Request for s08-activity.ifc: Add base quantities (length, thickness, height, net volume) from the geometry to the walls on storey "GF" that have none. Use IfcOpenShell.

First a look at what the model holds.

```python
import ifcopenshell
import ifcopenshell.util.element
import ifcopenshell.util.unit

model = ifcopenshell.open("s08-activity.ifc")
print(model.schema)
for unit_type in ("LENGTHUNIT", "AREAUNIT", "VOLUMEUNIT"):
    print(unit_type, ifcopenshell.util.unit.calculate_unit_scale(model, unit_type))
storey = next(s for s in model.by_type("IfcBuildingStorey") if s.Name == "GF")
walls = [e for e in ifcopenshell.util.element.get_decomposition(storey) if e.is_a("IfcWall")]
for e in sorted(walls, key=lambda e: e.id()):
    print(e.id(), e.is_a(), e.Name, list(ifcopenshell.util.element.get_psets(e, qtos_only=True)), sep=" | ")
```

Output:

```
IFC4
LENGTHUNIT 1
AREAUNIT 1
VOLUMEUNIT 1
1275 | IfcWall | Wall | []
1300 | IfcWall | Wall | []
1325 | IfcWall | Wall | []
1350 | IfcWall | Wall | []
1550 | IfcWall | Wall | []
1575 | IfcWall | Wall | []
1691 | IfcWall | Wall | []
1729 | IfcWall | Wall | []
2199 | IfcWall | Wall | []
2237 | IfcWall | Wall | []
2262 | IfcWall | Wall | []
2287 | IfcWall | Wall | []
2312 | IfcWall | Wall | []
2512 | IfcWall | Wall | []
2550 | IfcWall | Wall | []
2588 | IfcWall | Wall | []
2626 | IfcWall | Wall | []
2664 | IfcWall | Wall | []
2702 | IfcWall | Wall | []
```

```python
import ifcopenshell
import ifcopenshell.api.pset
import ifcopenshell.geom
import ifcopenshell.util.element
import ifcopenshell.util.shape
import ifcopenshell.util.unit

model = ifcopenshell.open("s08-activity.ifc")
unit_scale = ifcopenshell.util.unit.calculate_unit_scale(model)
volume_scale = ifcopenshell.util.unit.calculate_unit_scale(model, "VOLUMEUNIT")
settings = ifcopenshell.geom.settings()

storey = next(s for s in model.by_type("IfcBuildingStorey") if s.Name == "GF")
walls = [e for e in ifcopenshell.util.element.get_decomposition(storey) if e.is_a("IfcWall")]

for e in sorted(walls, key=lambda e: e.id()):
    if ifcopenshell.util.element.get_psets(e, qtos_only=True, should_inherit=False):
        continue
    # Geometry comes back in metres, in the element's own axes.
    shape = ifcopenshell.geom.create_shape(settings, e)
    values = {
        "Length": ifcopenshell.util.shape.get_x(shape.geometry) / unit_scale,
        "Width": ifcopenshell.util.shape.get_y(shape.geometry) / unit_scale,
        "Height": ifcopenshell.util.shape.get_z(shape.geometry) / unit_scale,
        "NetVolume": ifcopenshell.util.shape.get_volume(shape.geometry) / volume_scale,
    }
    qto = ifcopenshell.api.pset.add_qto(model, product=e, name="Qto_WallBaseQuantities")
    ifcopenshell.api.pset.edit_qto(model, qto=qto, properties=values)
    print(e.id(), {k: round(v, 3) for k, v in values.items()})

model.write("s08-activity_v2.ifc")
```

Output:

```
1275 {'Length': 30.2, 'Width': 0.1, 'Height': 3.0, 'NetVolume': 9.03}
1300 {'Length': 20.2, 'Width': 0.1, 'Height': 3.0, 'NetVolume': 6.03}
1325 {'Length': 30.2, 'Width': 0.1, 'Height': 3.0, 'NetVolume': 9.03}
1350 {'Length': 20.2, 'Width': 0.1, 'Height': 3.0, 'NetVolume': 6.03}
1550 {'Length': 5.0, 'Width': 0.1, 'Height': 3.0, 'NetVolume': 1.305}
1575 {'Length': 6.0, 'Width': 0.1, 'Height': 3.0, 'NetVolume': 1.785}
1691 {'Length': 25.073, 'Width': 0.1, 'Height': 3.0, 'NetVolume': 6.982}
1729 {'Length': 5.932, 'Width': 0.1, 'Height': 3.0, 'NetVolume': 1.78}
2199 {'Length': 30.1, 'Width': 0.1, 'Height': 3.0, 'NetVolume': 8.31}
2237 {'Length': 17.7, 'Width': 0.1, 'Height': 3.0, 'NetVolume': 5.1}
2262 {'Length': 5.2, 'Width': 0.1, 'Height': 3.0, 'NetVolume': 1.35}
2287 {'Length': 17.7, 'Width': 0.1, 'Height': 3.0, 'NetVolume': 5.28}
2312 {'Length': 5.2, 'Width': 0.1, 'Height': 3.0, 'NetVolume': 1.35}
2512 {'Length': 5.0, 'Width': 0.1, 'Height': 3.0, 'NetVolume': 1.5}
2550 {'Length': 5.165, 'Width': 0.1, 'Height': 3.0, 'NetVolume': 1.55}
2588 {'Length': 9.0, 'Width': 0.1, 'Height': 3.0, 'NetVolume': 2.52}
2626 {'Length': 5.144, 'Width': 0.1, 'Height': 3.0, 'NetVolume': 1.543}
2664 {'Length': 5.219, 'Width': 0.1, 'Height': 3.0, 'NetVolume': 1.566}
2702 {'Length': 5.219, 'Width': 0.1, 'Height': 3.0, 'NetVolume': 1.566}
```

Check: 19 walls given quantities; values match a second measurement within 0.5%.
